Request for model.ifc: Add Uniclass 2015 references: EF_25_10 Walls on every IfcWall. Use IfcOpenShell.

First a look at what the model holds.

```python
import ifcopenshell

model = ifcopenshell.open("model.ifc")
print(model.schema)
print("classifications:", [c.Name for c in model.by_type("IfcClassification")])
for ifc_class in ("IfcDoor", "IfcRoof", "IfcStair", "IfcWall", "IfcWindow"):
    print(ifc_class, len(model.by_type(ifc_class)))
```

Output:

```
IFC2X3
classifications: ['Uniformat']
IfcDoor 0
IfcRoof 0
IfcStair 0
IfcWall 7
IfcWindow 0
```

```python
import ifcopenshell
import ifcopenshell.api.classification

model = ifcopenshell.open("model.ifc")

# IFC2X3 requires Source and Edition and has no link from the project to the system.
system = model.create_entity("IfcClassification", Source="NBS", Edition="2015", Name="Uniclass 2015")

codes = {
    "IfcWall": ("EF_25_10", "Walls"),
}
for ifc_class, (code, name) in codes.items():
    products = model.by_type(ifc_class)
    ifcopenshell.api.classification.add_reference(
        model, products=products, classification=system, identification=code, name=name
    )
    print(code, len(products))

model.write("model_v2.ifc")
```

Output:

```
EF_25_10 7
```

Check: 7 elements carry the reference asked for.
